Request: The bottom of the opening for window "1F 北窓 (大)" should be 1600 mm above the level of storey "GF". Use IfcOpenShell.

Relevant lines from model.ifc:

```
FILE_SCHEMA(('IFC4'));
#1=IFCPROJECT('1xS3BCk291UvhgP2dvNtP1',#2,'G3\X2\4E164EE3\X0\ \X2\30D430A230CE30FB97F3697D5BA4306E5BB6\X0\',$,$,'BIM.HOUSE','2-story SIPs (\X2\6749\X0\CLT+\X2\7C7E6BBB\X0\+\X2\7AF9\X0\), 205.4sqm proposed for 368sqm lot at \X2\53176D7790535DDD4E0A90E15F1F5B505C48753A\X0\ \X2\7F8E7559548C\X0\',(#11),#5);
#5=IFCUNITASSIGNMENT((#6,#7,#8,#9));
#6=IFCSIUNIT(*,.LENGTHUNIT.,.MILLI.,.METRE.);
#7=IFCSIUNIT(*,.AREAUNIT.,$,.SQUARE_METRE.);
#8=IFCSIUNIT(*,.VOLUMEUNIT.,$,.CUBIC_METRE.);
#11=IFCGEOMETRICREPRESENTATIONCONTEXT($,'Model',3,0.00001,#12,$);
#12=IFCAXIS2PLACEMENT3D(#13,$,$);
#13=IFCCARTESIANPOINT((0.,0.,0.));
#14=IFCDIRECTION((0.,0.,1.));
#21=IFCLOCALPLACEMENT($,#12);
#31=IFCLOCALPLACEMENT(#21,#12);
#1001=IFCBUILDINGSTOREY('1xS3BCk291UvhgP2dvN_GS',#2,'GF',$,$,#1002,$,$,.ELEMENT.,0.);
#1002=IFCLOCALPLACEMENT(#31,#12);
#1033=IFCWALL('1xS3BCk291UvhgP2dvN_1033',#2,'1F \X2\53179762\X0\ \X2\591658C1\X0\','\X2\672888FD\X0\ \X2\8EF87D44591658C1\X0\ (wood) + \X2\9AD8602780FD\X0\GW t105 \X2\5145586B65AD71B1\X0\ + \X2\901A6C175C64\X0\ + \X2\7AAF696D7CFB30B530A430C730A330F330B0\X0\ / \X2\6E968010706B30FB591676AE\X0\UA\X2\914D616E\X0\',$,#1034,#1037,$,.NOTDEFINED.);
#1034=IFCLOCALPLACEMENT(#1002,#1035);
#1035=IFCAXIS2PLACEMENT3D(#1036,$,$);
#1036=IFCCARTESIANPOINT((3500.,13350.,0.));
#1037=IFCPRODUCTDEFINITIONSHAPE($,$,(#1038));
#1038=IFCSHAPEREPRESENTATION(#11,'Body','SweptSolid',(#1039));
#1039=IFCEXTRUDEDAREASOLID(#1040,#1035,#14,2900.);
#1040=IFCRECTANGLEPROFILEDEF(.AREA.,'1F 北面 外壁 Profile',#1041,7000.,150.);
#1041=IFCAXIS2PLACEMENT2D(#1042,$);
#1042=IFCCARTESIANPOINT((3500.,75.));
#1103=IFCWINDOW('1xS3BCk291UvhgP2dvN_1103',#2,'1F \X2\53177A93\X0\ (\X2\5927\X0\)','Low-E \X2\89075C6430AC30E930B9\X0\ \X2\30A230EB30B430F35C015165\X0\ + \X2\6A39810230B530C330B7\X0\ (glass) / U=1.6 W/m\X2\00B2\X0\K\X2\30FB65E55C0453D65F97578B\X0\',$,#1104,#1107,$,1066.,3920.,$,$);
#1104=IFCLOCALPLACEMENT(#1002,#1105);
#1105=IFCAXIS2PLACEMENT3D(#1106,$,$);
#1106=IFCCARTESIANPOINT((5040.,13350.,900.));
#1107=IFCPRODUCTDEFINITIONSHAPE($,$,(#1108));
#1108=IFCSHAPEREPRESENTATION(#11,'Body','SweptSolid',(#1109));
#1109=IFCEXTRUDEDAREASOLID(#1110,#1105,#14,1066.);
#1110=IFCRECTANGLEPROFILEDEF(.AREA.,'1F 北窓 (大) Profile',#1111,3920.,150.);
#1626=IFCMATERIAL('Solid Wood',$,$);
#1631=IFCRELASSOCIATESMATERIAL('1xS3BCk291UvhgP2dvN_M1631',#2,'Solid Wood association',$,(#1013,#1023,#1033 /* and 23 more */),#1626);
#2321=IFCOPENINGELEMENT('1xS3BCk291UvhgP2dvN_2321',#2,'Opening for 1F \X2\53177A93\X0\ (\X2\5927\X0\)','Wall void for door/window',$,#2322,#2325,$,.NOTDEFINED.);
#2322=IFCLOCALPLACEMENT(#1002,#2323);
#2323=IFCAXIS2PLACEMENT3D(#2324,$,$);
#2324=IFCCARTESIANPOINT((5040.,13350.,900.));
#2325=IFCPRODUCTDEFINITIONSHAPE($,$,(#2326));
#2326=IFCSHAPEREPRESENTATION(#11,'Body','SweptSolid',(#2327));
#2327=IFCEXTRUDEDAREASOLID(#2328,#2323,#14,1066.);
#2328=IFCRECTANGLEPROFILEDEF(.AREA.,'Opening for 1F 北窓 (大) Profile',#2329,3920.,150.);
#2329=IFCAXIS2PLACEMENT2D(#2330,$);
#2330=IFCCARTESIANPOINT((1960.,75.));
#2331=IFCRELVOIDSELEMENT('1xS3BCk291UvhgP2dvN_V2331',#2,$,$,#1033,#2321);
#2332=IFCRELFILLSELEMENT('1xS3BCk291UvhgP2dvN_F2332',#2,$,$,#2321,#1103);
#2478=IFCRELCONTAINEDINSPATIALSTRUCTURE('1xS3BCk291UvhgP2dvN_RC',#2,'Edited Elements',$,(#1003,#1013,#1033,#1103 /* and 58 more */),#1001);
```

```python
import numpy as np
import ifcopenshell
import ifcopenshell.api.geometry
import ifcopenshell.geom
import ifcopenshell.util.element
import ifcopenshell.util.placement
import ifcopenshell.util.shape
import ifcopenshell.util.unit

model = ifcopenshell.open("model.ifc")
unit_scale = ifcopenshell.util.unit.calculate_unit_scale(model)

window = model.by_guid("1xS3BCk291UvhgP2dvN_1103")
opening = window.FillsVoids[0].RelatingOpeningElement
storey = ifcopenshell.util.element.get_container(window, ifc_class="IfcBuildingStorey")
level = ifcopenshell.util.placement.get_local_placement(storey.ObjectPlacement)[2, 3]

# The opening's origin need not be at the sill, so measure its lowest point.
shape = ifcopenshell.geom.create_shape(ifcopenshell.geom.settings(), opening)
bottom = ifcopenshell.util.shape.get_shape_bottom_elevation(shape, shape.geometry) / unit_scale
dz = level + 1.6 / unit_scale - bottom

shift = np.array([0.0, 0.0, dz])
# The window is not placed relative to its opening, so move both.
for product in (opening, window):
    matrix = ifcopenshell.util.placement.get_local_placement(product.ObjectPlacement)
    matrix[:3, 3] += shift
    ifcopenshell.api.geometry.edit_object_placement(model, product=product, matrix=matrix, is_si=False)

print(f"moved by {dz * unit_scale:+.3f} m")

model.write("model-out.ifc")
```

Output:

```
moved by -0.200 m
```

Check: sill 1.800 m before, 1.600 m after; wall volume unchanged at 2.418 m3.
